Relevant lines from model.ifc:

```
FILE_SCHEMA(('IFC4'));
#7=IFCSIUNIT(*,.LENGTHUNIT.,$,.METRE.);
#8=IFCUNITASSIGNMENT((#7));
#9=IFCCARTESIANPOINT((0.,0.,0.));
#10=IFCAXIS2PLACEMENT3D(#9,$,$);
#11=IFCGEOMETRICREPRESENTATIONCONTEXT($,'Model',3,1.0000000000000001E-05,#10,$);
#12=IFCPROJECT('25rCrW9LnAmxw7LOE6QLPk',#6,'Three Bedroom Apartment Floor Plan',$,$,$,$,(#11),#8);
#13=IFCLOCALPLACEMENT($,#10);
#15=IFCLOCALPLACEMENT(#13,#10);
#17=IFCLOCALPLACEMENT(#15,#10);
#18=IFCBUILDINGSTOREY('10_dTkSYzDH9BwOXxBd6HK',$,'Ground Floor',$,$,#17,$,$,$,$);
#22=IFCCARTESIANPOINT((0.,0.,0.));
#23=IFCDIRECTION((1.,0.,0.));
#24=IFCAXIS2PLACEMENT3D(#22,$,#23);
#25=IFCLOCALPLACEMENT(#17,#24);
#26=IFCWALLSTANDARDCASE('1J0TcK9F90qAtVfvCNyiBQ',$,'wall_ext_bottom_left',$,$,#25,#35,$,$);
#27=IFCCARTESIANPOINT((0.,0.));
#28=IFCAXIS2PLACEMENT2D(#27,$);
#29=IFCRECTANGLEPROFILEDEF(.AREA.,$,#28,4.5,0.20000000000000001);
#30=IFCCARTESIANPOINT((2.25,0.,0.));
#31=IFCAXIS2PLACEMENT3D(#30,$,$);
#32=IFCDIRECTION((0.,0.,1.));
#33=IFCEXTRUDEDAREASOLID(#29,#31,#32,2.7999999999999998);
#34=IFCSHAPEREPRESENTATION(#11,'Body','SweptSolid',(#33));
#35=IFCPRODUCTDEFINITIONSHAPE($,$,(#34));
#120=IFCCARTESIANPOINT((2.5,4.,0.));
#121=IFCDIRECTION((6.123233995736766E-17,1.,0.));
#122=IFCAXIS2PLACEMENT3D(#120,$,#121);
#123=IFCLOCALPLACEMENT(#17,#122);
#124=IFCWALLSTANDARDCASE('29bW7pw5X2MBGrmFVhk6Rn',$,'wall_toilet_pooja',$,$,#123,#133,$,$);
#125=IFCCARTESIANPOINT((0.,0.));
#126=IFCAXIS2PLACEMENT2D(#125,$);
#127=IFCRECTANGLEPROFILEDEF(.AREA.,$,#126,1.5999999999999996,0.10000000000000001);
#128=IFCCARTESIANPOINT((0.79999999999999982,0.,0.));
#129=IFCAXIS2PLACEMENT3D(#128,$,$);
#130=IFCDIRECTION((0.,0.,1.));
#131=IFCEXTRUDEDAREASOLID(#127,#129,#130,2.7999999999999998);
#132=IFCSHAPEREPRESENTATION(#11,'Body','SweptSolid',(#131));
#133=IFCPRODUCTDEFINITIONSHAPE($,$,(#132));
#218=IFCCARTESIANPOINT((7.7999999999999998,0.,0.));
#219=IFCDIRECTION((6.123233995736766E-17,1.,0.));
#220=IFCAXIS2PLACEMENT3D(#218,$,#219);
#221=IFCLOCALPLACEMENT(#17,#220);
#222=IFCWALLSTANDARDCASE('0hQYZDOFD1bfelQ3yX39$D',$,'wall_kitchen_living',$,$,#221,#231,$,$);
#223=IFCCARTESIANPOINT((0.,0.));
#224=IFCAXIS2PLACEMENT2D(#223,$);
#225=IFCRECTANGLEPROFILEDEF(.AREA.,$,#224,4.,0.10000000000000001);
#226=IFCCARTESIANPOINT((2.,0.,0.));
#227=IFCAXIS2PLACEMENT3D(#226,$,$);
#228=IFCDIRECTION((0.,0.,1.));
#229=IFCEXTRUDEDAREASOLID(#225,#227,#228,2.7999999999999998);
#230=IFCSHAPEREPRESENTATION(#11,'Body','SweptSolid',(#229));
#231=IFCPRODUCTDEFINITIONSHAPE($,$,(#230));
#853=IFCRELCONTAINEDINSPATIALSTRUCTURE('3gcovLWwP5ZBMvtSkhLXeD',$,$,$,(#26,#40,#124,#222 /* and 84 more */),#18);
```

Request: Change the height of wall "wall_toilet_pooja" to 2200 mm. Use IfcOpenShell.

```python
import ifcopenshell
import ifcopenshell.geom
import ifcopenshell.util.shape
import ifcopenshell.util.unit

model = ifcopenshell.open("model.ifc")
unit_scale = ifcopenshell.util.unit.calculate_unit_scale(model)
settings = ifcopenshell.geom.settings()


def volume(element):
    """Net volume in cubic metres, openings subtracted."""
    shape = ifcopenshell.geom.create_shape(settings, element)
    return ifcopenshell.util.shape.get_volume(shape.geometry)


wall = model.by_id(124)
before = volume(wall)

body = next(r for r in wall.Representation.Representations if r.RepresentationIdentifier == "Body")
solid = body.Items[0]
old_height = solid.Depth
solid.Depth = 2.2 / unit_scale
after = volume(wall)

print(f"height {old_height:g} -> {solid.Depth:g}, volume {before:.3f} -> {after:.3f} m3")

model.write("model-out.ifc")
```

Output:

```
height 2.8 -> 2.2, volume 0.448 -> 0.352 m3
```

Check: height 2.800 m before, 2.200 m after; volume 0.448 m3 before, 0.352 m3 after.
